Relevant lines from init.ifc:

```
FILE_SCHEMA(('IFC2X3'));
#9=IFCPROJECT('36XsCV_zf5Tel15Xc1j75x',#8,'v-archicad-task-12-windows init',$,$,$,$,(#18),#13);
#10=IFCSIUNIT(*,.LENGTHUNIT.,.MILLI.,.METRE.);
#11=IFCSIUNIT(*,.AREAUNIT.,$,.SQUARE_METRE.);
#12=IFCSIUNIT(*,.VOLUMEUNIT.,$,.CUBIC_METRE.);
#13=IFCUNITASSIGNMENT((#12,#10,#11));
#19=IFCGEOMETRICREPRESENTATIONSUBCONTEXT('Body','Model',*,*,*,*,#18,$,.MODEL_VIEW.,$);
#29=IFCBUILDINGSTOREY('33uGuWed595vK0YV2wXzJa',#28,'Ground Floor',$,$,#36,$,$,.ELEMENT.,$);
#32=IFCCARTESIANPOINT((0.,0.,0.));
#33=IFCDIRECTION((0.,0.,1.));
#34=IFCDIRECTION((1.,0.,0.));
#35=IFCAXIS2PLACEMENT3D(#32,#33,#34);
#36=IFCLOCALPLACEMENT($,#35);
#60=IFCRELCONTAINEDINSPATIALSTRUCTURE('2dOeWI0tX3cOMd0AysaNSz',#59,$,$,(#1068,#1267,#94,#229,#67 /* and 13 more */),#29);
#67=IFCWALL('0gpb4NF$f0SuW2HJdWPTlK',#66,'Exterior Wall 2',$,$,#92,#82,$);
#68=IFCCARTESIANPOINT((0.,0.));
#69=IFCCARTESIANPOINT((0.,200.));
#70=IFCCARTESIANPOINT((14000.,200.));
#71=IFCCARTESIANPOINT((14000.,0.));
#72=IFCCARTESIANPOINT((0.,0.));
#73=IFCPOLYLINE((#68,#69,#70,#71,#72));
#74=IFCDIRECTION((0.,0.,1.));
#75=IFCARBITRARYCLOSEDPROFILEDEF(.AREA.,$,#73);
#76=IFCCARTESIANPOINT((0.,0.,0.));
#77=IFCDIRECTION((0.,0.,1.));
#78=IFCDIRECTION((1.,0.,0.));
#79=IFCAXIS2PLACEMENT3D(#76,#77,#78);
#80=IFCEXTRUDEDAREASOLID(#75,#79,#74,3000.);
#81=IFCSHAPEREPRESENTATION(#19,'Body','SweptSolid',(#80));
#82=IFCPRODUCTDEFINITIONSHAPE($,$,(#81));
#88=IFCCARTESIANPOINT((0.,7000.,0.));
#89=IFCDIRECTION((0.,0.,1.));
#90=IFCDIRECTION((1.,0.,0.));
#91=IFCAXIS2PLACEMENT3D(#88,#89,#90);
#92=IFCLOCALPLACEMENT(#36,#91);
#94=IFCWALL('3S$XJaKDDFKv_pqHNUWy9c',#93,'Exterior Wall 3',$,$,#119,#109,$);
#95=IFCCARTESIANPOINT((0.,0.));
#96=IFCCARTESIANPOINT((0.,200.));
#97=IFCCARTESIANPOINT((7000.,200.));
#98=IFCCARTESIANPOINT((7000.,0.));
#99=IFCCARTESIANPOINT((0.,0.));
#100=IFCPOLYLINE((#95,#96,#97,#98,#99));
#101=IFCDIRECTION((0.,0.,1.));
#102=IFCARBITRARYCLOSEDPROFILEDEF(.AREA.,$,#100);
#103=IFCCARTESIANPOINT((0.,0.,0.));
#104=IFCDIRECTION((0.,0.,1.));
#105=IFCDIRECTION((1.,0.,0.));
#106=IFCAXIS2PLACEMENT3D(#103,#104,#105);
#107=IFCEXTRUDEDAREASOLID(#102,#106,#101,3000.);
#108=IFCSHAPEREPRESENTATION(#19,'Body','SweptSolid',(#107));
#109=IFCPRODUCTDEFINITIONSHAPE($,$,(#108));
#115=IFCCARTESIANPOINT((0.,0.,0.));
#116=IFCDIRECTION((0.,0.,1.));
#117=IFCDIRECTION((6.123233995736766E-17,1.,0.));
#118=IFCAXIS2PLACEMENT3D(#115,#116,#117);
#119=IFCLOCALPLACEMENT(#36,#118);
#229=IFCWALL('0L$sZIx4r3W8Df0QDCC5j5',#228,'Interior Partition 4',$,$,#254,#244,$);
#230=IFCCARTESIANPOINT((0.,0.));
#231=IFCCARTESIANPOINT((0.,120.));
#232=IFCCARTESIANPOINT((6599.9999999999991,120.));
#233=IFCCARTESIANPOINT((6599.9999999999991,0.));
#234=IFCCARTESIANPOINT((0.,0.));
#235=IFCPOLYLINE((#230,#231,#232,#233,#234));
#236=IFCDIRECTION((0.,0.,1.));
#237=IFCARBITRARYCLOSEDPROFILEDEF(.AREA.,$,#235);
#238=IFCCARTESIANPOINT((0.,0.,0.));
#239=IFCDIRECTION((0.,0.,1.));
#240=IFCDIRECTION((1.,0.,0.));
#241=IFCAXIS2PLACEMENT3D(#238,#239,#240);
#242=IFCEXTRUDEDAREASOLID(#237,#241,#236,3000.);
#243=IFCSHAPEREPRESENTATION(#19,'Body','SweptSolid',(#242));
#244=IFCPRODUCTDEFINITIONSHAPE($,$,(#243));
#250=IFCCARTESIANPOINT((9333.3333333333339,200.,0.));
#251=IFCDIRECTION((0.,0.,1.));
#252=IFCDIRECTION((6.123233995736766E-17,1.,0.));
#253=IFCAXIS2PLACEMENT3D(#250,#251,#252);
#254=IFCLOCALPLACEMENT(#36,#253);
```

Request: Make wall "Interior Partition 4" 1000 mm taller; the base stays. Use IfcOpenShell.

```python
import ifcopenshell
import ifcopenshell.geom
import ifcopenshell.util.representation
import ifcopenshell.util.shape

model = ifcopenshell.open("init.ifc")
settings = ifcopenshell.geom.settings()


def volume(element):
    """Net volume in cubic metres, openings subtracted."""
    shape = ifcopenshell.geom.create_shape(settings, element)
    return ifcopenshell.util.shape.get_volume(shape.geometry)


wall = model.by_guid("0L$sZIx4r3W8Df0QDCC5j5")
before = volume(wall)

body = ifcopenshell.util.representation.get_representation(wall, "Model", "Body")
solid = body.Items[0]
old_height = solid.Depth
solid.Depth += 1000.0
after = volume(wall)

print(f"height {old_height:g} -> {solid.Depth:g}, volume {before:.3f} -> {after:.3f} m3")

model.write("init_updated.ifc")
```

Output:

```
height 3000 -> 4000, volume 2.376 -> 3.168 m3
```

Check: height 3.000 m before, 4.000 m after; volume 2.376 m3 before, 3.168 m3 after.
